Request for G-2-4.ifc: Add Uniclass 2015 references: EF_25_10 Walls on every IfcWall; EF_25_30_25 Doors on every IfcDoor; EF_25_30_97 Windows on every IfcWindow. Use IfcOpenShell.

First a look at what the model holds.

```python
import ifcopenshell

model = ifcopenshell.open("G-2-4.ifc")
print(model.schema)
print("classifications:", [c.Name for c in model.by_type("IfcClassification")])
for ifc_class in ("IfcDoor", "IfcRoof", "IfcStair", "IfcWall", "IfcWindow"):
    print(ifc_class, len(model.by_type(ifc_class)))
```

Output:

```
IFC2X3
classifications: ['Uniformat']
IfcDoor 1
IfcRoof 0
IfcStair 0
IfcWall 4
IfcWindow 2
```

```python
import ifcopenshell
import ifcopenshell.api.classification

model = ifcopenshell.open("G-2-4.ifc")

# IFC2X3 requires Source and Edition and has no link from the project to the system.
system = model.create_entity("IfcClassification", Source="NBS", Edition="2015", Name="Uniclass 2015")

codes = {
    "IfcWall": ("EF_25_10", "Walls"),
    "IfcDoor": ("EF_25_30_25", "Doors"),
    "IfcWindow": ("EF_25_30_97", "Windows"),
}
for ifc_class, (code, name) in codes.items():
    products = model.by_type(ifc_class)
    ifcopenshell.api.classification.add_reference(
        model, products=products, classification=system, identification=code, name=name
    )
    print(code, len(products))

model.write("G-2-4_edited.ifc")
```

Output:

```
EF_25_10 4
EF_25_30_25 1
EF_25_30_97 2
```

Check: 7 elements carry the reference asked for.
